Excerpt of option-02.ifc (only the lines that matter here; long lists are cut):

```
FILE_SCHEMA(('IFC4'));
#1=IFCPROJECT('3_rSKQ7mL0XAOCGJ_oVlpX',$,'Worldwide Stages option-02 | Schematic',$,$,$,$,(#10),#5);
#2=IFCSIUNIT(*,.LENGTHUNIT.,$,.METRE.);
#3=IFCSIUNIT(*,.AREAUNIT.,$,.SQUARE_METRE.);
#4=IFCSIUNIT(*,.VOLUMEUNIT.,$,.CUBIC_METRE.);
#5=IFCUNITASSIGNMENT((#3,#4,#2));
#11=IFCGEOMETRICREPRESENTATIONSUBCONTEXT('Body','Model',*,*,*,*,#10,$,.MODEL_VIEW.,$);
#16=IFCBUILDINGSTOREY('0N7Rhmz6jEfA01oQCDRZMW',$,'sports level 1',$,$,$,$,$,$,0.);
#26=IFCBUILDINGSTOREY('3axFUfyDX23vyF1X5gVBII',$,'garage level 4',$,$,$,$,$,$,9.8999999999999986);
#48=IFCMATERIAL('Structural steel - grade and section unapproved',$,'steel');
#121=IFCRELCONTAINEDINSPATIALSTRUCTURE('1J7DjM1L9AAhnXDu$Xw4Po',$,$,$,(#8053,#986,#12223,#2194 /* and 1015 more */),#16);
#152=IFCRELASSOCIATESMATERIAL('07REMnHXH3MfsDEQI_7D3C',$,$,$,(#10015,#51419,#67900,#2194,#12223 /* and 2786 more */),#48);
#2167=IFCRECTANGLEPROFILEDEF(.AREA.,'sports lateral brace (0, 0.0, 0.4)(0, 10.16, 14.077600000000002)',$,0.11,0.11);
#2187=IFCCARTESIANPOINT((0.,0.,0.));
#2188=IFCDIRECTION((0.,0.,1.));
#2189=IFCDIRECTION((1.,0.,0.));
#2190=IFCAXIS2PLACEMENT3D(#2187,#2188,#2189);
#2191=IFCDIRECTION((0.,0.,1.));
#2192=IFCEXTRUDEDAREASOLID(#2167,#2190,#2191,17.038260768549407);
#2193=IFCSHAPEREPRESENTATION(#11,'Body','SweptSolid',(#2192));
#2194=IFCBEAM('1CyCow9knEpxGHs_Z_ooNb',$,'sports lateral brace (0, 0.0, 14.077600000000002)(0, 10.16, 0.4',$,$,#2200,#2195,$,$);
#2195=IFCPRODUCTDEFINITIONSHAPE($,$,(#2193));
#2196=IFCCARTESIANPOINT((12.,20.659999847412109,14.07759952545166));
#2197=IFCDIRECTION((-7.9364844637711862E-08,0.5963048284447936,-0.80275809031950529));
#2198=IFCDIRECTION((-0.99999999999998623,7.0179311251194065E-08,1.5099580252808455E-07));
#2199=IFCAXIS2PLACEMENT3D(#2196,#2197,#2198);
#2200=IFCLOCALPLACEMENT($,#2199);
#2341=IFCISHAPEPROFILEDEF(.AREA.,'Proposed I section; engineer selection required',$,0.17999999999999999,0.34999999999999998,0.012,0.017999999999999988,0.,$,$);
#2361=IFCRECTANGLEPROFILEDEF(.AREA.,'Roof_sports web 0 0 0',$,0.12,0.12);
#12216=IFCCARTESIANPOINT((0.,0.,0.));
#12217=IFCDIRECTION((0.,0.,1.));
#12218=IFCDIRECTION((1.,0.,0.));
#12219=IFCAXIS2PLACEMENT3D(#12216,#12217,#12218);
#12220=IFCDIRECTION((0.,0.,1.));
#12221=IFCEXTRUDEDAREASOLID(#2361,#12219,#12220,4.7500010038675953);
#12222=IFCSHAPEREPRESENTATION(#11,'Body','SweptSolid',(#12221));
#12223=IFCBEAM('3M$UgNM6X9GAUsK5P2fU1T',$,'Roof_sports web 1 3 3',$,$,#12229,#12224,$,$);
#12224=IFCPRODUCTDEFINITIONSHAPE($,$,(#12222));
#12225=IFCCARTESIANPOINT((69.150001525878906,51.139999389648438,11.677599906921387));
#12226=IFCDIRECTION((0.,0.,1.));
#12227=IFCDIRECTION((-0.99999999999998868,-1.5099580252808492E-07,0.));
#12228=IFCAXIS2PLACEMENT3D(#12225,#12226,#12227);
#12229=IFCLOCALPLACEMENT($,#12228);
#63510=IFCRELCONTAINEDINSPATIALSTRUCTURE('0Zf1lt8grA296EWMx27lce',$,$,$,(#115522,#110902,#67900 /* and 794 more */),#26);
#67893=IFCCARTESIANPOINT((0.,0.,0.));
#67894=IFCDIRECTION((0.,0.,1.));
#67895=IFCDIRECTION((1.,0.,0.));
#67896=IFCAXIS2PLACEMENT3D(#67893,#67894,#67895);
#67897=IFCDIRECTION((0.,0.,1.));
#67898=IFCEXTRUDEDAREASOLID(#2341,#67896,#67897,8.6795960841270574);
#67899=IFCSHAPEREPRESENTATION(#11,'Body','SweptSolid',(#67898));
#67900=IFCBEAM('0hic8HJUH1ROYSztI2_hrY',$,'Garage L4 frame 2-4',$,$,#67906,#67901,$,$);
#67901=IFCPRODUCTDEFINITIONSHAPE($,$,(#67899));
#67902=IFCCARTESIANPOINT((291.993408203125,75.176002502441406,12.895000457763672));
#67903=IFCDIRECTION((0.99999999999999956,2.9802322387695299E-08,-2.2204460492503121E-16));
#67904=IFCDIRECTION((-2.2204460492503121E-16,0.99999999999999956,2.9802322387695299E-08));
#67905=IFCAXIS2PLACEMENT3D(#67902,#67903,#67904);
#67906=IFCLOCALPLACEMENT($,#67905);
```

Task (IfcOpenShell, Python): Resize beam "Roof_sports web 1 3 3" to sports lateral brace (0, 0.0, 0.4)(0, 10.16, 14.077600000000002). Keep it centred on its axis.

```python
import ifcopenshell
import ifcopenshell.util.element
import ifcopenshell.util.representation

model = ifcopenshell.open("option-02.ifc")

member = model.by_guid("3M$UgNM6X9GAUsK5P2fU1T")
source = next(p for p in model.by_type("IfcRectangleProfileDef") if p.ProfileName == "sports lateral brace (0, 0.0, 0.4)(0, 10.16, 14.077600000000002)")

body = ifcopenshell.util.representation.get_representation(member, "Model", "Body")
solid = body.Items[0]
old_profile = solid.SweptArea

# Copy the section's sizes but keep this member's own profile position.
profile = ifcopenshell.util.element.copy(model, source)
profile.Position = old_profile.Position
solid.SweptArea = profile
if not model.get_total_inverses(old_profile):
    ifcopenshell.util.element.remove_deep2(model, old_profile)

print(solid.SweptArea)

model.write("option-02_rev.ifc")
```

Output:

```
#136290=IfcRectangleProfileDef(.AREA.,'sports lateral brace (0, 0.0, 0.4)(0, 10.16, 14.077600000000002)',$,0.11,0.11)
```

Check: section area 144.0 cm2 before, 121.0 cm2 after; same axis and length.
